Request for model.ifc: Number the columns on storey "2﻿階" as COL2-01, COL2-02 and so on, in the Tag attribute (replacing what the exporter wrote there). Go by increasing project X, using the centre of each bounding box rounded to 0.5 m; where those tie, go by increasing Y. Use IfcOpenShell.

First a look at what the model holds.

```python
import ifcopenshell
import ifcopenshell.util.element
import ifcopenshell.util.placement

model = ifcopenshell.open("model.ifc")
print(model.schema)
storey = next(s for s in model.by_type("IfcBuildingStorey") if s.Name == '2\ufeff階')
columns = [e for e in ifcopenshell.util.element.get_decomposition(storey) if e.is_a("IfcColumn")]
for e in sorted(columns, key=lambda e: e.id()):
    origin = ifcopenshell.util.placement.get_local_placement(e.ObjectPlacement)[:3, 3]
    print(e.id(), e.Tag, e.Name, origin.round(2) + 0.0, sep=" | ")
```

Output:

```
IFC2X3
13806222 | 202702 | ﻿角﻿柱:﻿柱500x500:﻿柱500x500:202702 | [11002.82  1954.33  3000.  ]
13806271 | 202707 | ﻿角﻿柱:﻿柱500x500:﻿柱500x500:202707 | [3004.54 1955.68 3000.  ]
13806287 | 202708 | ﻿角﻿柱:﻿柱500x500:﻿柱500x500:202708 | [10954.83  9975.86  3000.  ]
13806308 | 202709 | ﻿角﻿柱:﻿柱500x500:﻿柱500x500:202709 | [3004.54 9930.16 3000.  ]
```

```python
import ifcopenshell
import ifcopenshell.geom
import ifcopenshell.util.element
import ifcopenshell.util.shape

model = ifcopenshell.open("model.ifc")
settings = ifcopenshell.geom.settings()
settings.set("use-world-coords", True)


def centre(element):
    shape = ifcopenshell.geom.create_shape(settings, element)
    return ifcopenshell.util.shape.get_bbox_centroid(shape.geometry)


storey = next(s for s in model.by_type("IfcBuildingStorey") if s.Name == '2\ufeff階')
columns = [e for e in ifcopenshell.util.element.get_decomposition(storey) if e.is_a("IfcColumn")]

# Insertion points can sit at a corner or the storey origin, so sort by the geometry (in metres).
centres = {e: centre(e) for e in columns}
columns.sort(key=lambda e: (round(centres[e][0] / 0.5), centres[e][1]))

for i, e in enumerate(columns, start=1):
    number = f"COL2-{i:02d}"
    e.Tag = number
    print(e.id(), number)

model.write("model-out.ifc")
```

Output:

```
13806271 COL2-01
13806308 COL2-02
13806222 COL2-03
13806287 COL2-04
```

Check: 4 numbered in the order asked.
